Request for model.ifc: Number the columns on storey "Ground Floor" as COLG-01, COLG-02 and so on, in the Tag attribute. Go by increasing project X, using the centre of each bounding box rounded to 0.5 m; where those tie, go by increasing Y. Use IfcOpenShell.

First a look at what the model holds.

```python
import ifcopenshell
import ifcopenshell.util.element
import ifcopenshell.util.placement

model = ifcopenshell.open("model.ifc")
print(model.schema)
storey = next(s for s in model.by_type("IfcBuildingStorey") if s.Name == "Ground Floor")
columns = [e for e in ifcopenshell.util.element.get_decomposition(storey) if e.is_a("IfcColumn")]
for e in sorted(columns, key=lambda e: e.id()):
    origin = ifcopenshell.util.placement.get_local_placement(e.ObjectPlacement)[:3, 3]
    print(e.id(), e.Tag, e.Name, origin.round(2) + 0.0, sep=" | ")
```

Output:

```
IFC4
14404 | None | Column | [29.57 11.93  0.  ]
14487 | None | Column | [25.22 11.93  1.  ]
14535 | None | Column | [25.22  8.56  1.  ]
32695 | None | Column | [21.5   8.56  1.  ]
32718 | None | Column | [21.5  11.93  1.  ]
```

```python
import ifcopenshell
import ifcopenshell.geom
import ifcopenshell.util.element
import ifcopenshell.util.shape

model = ifcopenshell.open("model.ifc")
settings = ifcopenshell.geom.settings()
settings.set("use-world-coords", True)


def centre(element):
    shape = ifcopenshell.geom.create_shape(settings, element)
    return ifcopenshell.util.shape.get_bbox_centroid(shape.geometry)


storey = next(s for s in model.by_type("IfcBuildingStorey") if s.Name == "Ground Floor")
columns = [e for e in ifcopenshell.util.element.get_decomposition(storey) if e.is_a("IfcColumn")]

# Insertion points can sit at a corner or the storey origin, so sort by the geometry (in metres).
centres = {e: centre(e) for e in columns}
columns.sort(key=lambda e: (round(centres[e][0] / 0.5), centres[e][1]))

for i, e in enumerate(columns, start=1):
    number = f"COLG-{i:02d}"
    e.Tag = number
    print(e.id(), number)

model.write("model-out.ifc")
```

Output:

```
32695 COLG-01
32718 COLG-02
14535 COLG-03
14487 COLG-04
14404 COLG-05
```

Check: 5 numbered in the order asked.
